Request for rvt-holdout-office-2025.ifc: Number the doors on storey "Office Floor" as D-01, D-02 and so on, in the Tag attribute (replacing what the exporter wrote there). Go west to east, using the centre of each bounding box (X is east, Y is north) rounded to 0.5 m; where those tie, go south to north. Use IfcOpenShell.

First a look at what the model holds.

```python
import ifcopenshell
import ifcopenshell.util.element
import ifcopenshell.util.placement

model = ifcopenshell.open("rvt-holdout-office-2025.ifc")
print(model.schema)
storey = next(s for s in model.by_type("IfcBuildingStorey") if s.Name == "Office Floor")
doors = [e for e in ifcopenshell.util.element.get_decomposition(storey) if e.is_a("IfcDoor")]
for e in sorted(doors, key=lambda e: e.id()):
    origin = ifcopenshell.util.placement.get_local_placement(e.ObjectPlacement)[:3, 3]
    print(e.id(), e.Tag, e.Name, origin.round(2) + 0.0, sep=" | ")
```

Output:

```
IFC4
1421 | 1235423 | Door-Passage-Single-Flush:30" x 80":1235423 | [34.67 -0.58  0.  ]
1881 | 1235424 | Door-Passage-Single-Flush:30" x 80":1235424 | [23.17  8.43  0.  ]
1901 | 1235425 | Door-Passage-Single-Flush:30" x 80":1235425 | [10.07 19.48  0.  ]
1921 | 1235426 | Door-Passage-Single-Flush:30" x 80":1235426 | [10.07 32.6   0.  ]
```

```python
import ifcopenshell
import ifcopenshell.geom
import ifcopenshell.util.element
import ifcopenshell.util.shape

model = ifcopenshell.open("rvt-holdout-office-2025.ifc")
settings = ifcopenshell.geom.settings()
settings.set("use-world-coords", True)


def centre(element):
    shape = ifcopenshell.geom.create_shape(settings, element)
    return ifcopenshell.util.shape.get_bbox_centroid(shape.geometry)


storey = next(s for s in model.by_type("IfcBuildingStorey") if s.Name == "Office Floor")
doors = [e for e in ifcopenshell.util.element.get_decomposition(storey) if e.is_a("IfcDoor")]

# Insertion points can sit at a corner or the storey origin, so sort by the geometry (in metres).
centres = {e: centre(e) for e in doors}
doors.sort(key=lambda e: (round(centres[e][0] / 0.5), centres[e][1]))

for i, e in enumerate(doors, start=1):
    number = f"D-{i:02d}"
    e.Tag = number
    print(e.id(), number)

model.write("rvt-holdout-office-2025_v2.ifc")
```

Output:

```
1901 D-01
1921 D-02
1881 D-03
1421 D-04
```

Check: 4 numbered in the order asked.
